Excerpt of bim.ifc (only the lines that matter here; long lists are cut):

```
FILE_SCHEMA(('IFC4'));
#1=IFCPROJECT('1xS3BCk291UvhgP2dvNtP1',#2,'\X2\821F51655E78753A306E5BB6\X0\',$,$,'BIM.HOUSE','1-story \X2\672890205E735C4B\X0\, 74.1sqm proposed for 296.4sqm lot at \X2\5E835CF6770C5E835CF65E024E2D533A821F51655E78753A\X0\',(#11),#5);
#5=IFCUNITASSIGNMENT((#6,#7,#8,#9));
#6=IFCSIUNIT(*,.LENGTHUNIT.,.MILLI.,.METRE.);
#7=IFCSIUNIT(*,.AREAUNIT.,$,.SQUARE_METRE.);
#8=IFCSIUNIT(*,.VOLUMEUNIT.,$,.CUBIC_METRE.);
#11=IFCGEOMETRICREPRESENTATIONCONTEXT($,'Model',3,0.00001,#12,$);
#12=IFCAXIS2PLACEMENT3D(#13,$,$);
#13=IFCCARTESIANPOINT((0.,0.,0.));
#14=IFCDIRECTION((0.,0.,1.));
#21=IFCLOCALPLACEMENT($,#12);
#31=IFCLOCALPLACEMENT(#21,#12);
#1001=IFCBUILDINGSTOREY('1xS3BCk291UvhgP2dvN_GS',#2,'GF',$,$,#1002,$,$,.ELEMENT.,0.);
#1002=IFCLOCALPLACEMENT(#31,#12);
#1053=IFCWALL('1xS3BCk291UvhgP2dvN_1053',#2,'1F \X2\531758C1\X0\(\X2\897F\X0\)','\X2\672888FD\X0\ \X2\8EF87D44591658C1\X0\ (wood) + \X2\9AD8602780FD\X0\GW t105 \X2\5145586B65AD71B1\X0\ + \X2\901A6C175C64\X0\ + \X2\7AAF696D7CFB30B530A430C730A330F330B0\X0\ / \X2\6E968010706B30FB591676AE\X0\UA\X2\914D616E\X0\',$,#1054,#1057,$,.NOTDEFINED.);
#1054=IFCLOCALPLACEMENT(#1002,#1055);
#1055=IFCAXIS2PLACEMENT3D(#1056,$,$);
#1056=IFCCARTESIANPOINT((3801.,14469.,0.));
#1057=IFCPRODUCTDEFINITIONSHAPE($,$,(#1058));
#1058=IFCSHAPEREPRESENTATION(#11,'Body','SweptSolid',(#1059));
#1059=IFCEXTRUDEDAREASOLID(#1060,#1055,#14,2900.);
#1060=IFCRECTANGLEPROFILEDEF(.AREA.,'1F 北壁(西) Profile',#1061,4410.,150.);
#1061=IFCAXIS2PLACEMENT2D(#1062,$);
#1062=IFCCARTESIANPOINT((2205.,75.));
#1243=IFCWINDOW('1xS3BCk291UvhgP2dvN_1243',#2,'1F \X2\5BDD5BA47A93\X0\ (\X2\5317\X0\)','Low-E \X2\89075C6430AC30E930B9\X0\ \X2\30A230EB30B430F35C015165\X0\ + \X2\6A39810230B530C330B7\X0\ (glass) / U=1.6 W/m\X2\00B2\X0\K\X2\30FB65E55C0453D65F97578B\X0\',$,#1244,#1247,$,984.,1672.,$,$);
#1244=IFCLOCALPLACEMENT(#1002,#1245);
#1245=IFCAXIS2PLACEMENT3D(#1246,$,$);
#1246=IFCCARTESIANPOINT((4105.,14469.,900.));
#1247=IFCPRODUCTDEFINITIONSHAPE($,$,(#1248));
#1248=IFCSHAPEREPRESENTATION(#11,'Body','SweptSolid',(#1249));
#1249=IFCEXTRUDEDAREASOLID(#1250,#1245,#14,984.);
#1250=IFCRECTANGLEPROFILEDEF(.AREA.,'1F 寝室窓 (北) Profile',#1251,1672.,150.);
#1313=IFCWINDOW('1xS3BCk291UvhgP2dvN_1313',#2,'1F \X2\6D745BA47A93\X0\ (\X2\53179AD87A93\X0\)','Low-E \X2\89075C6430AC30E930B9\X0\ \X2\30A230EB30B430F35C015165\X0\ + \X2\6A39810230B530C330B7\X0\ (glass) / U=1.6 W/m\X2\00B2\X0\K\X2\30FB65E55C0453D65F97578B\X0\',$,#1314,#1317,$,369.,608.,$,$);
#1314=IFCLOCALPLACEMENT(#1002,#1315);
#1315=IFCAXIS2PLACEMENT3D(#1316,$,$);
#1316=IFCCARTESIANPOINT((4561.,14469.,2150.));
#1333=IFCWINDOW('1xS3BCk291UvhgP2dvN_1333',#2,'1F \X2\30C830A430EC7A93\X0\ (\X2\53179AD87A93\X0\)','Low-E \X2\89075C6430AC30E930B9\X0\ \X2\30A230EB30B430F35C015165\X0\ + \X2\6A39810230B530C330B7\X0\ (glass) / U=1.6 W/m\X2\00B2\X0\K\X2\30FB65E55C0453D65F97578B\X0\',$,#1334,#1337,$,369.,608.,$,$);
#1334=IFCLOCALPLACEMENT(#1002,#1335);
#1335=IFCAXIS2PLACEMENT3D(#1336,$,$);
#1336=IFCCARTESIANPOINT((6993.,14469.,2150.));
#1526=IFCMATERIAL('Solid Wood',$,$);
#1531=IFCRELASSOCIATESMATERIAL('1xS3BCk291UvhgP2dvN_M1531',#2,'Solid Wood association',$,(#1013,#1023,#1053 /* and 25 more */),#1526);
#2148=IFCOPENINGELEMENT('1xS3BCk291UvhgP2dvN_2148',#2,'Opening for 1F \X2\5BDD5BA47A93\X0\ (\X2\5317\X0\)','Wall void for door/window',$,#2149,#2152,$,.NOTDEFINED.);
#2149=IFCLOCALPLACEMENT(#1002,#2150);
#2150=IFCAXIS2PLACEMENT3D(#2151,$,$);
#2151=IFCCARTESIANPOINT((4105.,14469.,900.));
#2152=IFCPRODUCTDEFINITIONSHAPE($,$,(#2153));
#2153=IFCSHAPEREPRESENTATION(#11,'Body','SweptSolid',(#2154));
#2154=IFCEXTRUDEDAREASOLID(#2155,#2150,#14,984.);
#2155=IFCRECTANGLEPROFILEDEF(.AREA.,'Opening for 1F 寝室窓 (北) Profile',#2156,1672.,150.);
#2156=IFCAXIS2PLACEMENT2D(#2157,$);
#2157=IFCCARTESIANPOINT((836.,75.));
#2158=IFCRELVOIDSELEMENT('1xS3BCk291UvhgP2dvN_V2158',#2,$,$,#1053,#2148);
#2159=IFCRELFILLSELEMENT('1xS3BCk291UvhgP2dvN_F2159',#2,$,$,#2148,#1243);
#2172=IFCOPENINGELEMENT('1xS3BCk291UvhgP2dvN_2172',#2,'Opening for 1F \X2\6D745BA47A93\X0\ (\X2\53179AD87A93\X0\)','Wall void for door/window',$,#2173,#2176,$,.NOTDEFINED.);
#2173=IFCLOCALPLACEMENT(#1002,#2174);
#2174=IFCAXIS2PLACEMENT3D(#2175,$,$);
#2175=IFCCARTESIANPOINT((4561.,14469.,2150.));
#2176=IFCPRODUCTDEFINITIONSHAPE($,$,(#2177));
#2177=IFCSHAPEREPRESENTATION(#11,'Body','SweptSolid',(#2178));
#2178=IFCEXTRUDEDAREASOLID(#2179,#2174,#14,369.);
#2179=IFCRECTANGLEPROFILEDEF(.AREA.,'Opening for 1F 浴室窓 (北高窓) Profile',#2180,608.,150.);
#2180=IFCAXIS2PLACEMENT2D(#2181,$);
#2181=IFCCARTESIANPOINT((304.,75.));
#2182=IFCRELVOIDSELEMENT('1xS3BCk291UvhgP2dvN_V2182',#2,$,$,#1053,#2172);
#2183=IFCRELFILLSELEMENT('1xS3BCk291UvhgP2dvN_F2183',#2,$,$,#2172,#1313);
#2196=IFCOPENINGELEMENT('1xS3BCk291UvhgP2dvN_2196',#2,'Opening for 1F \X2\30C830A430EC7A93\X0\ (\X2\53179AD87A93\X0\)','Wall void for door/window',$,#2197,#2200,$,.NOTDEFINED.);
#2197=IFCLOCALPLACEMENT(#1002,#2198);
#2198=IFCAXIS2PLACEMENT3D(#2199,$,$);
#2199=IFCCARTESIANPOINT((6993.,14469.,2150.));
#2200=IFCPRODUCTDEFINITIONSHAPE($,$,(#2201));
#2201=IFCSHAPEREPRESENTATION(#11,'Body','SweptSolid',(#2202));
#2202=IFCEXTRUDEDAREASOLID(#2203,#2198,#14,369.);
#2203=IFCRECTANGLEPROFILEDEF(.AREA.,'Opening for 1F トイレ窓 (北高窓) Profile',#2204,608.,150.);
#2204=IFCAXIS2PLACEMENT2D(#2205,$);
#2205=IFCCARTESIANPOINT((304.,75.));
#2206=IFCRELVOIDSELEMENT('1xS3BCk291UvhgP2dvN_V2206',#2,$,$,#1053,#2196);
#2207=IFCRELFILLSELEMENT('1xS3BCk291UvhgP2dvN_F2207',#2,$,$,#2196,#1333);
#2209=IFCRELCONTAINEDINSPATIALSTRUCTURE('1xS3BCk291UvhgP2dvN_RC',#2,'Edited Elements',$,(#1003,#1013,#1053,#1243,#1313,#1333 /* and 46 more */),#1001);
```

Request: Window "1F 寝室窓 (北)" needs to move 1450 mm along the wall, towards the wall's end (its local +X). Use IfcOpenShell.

```python
import ifcopenshell
import ifcopenshell.api.geometry
import ifcopenshell.util.placement
import ifcopenshell.util.unit

model = ifcopenshell.open("bim.ifc")
unit_scale = ifcopenshell.util.unit.calculate_unit_scale(model)

window = model.by_guid("1xS3BCk291UvhgP2dvN_1243")
opening = window.FillsVoids[0].RelatingOpeningElement
wall = opening.VoidsElements[0].RelatingBuildingElement

wall_matrix = ifcopenshell.util.placement.get_local_placement(wall.ObjectPlacement)
shift = wall_matrix[:3, 0] * 1.45 / unit_scale
before = ifcopenshell.util.placement.get_local_placement(window.ObjectPlacement)[:3, 3].copy()

# The window is not placed relative to its opening, so move both.
for product in (opening, window):
    matrix = ifcopenshell.util.placement.get_local_placement(product.ObjectPlacement)
    matrix[:3, 3] += shift
    ifcopenshell.api.geometry.edit_object_placement(model, product=product, matrix=matrix, is_si=False)

after = ifcopenshell.util.placement.get_local_placement(window.ObjectPlacement)[:3, 3]
print("window moved by", (after - before).round(3) + 0.0)

model.write("bim_v2.ifc")
```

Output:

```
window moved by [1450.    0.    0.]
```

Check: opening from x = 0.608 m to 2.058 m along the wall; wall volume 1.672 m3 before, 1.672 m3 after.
